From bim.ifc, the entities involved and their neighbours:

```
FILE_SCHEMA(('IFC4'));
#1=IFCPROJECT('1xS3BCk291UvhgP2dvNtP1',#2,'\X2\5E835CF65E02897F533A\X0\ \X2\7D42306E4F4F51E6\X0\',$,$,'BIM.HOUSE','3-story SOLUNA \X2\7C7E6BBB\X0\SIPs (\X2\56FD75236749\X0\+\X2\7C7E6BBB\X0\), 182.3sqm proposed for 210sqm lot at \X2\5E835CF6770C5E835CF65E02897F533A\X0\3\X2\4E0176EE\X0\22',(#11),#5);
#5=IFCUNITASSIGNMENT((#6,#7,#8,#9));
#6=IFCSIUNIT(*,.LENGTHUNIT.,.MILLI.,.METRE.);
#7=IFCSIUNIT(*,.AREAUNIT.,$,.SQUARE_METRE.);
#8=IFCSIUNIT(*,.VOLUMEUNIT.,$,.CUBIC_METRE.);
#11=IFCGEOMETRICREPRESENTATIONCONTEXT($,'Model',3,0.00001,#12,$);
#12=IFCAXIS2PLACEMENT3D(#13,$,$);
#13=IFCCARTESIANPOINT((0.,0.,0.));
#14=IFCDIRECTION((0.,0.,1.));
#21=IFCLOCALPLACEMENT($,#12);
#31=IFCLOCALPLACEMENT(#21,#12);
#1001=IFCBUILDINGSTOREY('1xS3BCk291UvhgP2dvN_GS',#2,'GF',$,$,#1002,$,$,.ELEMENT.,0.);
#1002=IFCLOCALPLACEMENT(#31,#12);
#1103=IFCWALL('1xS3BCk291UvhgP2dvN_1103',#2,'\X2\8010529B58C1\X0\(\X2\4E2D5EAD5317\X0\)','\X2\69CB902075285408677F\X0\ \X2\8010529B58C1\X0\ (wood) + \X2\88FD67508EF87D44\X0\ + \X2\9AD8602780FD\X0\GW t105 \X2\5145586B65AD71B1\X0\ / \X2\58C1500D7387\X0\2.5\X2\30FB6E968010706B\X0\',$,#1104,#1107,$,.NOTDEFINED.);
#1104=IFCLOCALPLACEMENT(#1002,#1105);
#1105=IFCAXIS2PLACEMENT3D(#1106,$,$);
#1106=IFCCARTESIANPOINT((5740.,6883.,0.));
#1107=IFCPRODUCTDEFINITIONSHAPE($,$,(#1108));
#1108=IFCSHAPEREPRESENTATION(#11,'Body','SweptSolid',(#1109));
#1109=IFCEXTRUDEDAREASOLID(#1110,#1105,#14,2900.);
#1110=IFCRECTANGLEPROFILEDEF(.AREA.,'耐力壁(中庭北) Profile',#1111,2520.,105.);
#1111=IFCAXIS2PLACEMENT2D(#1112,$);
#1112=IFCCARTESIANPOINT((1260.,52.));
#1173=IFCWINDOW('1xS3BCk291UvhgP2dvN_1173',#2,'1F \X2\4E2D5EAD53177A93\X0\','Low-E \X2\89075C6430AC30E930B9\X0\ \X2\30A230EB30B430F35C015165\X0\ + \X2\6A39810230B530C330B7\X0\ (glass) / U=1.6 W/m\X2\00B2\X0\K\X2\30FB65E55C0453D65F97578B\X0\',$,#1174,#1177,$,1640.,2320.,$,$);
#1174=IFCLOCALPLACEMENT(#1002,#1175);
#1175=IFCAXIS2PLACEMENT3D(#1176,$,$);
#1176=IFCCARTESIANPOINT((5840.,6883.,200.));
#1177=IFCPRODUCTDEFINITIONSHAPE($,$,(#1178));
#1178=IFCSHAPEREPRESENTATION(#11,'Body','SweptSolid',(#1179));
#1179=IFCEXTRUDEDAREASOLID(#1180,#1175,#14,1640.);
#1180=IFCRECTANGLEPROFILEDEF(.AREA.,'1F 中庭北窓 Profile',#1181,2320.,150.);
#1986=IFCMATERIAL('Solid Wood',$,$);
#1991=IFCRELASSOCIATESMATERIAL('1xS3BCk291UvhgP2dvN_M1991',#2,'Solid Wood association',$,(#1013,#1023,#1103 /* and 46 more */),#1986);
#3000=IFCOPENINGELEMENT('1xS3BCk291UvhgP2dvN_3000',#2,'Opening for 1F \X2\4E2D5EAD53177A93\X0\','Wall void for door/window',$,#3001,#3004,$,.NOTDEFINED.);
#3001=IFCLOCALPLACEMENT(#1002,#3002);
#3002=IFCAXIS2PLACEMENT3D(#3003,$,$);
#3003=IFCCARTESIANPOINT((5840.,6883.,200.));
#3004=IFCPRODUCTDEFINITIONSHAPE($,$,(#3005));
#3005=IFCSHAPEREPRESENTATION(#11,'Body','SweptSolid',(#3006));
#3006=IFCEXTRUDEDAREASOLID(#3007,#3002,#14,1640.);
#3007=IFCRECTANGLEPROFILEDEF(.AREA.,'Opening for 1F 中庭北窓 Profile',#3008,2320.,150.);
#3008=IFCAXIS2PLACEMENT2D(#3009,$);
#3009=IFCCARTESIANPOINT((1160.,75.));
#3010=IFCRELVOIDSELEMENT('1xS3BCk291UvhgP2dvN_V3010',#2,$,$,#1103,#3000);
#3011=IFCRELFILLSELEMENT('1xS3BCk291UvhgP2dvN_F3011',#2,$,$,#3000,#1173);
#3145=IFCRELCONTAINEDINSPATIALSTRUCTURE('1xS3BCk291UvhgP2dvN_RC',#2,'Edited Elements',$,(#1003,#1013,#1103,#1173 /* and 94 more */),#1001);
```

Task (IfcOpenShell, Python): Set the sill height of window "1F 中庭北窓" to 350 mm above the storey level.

```python
import numpy as np
import ifcopenshell
import ifcopenshell.api.geometry
import ifcopenshell.geom
import ifcopenshell.util.element
import ifcopenshell.util.placement
import ifcopenshell.util.shape
import ifcopenshell.util.unit

model = ifcopenshell.open("bim.ifc")
unit_scale = ifcopenshell.util.unit.calculate_unit_scale(model)

window = model.by_guid("1xS3BCk291UvhgP2dvN_1173")
opening = window.FillsVoids[0].RelatingOpeningElement
storey = ifcopenshell.util.element.get_container(window, ifc_class="IfcBuildingStorey")
level = ifcopenshell.util.placement.get_local_placement(storey.ObjectPlacement)[2, 3]

# The opening's origin need not be at the sill, so measure its lowest point.
shape = ifcopenshell.geom.create_shape(ifcopenshell.geom.settings(), opening)
bottom = ifcopenshell.util.shape.get_shape_bottom_elevation(shape, shape.geometry) / unit_scale
dz = level + 0.35 / unit_scale - bottom

shift = np.array([0.0, 0.0, dz])
# The window is not placed relative to its opening, so move both.
for product in (opening, window):
    matrix = ifcopenshell.util.placement.get_local_placement(product.ObjectPlacement)
    matrix[:3, 3] += shift
    ifcopenshell.api.geometry.edit_object_placement(model, product=product, matrix=matrix, is_si=False)

print(f"moved by {dz * unit_scale:+.3f} m")

model.write("bim-out.ifc")
```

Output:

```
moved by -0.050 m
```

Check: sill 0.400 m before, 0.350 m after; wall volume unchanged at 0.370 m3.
